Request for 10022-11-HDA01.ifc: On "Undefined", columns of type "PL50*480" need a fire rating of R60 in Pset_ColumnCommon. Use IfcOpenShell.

First a look at what the model holds.

```python
import ifcopenshell
import ifcopenshell.util.element

model = ifcopenshell.open("10022-11-HDA01.ifc")
print(model.schema)
storey = next(s for s in model.by_type("IfcBuildingStorey") if s.Name == "Undefined")
columns = [e for e in ifcopenshell.util.element.get_decomposition(storey) if e.is_a("IfcColumn")]
seen = {}
for e in columns:
    element_type = ifcopenshell.util.element.get_type(e)
    key = (element_type.Name if element_type != e and element_type else None, ifcopenshell.util.element.get_pset(e, "Pset_ColumnCommon", "FireRating"))
    seen[key] = seen.get(key, 0) + 1
for (name, value), count in sorted(seen.items(), key=str):
    print(count, "x", name, "|", value)
```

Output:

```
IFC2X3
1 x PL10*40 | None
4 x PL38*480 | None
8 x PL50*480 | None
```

```python
import ifcopenshell
import ifcopenshell.api.pset
import ifcopenshell.util.element

model = ifcopenshell.open("10022-11-HDA01.ifc")

storey = next(s for s in model.by_type("IfcBuildingStorey") if s.Name == "Undefined")
columns = [e for e in ifcopenshell.util.element.get_decomposition(storey) if e.is_a("IfcColumn")]

count = 0
for e in columns:
    element_type = ifcopenshell.util.element.get_type(e)
    if element_type in (None, e) or element_type.Name != "PL50*480":
        continue
    found = ifcopenshell.util.element.get_pset(e, "Pset_ColumnCommon", should_inherit=False)
    if found:
        pset = model.by_id(found["id"])
        if len(ifcopenshell.util.element.get_elements_by_pset(pset)) > 1:
            pset = ifcopenshell.api.pset.unshare_pset(model, products=[e], pset=pset)[0]
    else:
        pset = ifcopenshell.api.pset.add_pset(model, product=e, name="Pset_ColumnCommon")
    ifcopenshell.api.pset.edit_pset(model, pset=pset, properties={"FireRating": "R60"})
    count += 1

print(count, "columns updated")

model.write("10022-11-HDA01_edited.ifc")
```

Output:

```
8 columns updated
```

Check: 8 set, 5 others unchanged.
